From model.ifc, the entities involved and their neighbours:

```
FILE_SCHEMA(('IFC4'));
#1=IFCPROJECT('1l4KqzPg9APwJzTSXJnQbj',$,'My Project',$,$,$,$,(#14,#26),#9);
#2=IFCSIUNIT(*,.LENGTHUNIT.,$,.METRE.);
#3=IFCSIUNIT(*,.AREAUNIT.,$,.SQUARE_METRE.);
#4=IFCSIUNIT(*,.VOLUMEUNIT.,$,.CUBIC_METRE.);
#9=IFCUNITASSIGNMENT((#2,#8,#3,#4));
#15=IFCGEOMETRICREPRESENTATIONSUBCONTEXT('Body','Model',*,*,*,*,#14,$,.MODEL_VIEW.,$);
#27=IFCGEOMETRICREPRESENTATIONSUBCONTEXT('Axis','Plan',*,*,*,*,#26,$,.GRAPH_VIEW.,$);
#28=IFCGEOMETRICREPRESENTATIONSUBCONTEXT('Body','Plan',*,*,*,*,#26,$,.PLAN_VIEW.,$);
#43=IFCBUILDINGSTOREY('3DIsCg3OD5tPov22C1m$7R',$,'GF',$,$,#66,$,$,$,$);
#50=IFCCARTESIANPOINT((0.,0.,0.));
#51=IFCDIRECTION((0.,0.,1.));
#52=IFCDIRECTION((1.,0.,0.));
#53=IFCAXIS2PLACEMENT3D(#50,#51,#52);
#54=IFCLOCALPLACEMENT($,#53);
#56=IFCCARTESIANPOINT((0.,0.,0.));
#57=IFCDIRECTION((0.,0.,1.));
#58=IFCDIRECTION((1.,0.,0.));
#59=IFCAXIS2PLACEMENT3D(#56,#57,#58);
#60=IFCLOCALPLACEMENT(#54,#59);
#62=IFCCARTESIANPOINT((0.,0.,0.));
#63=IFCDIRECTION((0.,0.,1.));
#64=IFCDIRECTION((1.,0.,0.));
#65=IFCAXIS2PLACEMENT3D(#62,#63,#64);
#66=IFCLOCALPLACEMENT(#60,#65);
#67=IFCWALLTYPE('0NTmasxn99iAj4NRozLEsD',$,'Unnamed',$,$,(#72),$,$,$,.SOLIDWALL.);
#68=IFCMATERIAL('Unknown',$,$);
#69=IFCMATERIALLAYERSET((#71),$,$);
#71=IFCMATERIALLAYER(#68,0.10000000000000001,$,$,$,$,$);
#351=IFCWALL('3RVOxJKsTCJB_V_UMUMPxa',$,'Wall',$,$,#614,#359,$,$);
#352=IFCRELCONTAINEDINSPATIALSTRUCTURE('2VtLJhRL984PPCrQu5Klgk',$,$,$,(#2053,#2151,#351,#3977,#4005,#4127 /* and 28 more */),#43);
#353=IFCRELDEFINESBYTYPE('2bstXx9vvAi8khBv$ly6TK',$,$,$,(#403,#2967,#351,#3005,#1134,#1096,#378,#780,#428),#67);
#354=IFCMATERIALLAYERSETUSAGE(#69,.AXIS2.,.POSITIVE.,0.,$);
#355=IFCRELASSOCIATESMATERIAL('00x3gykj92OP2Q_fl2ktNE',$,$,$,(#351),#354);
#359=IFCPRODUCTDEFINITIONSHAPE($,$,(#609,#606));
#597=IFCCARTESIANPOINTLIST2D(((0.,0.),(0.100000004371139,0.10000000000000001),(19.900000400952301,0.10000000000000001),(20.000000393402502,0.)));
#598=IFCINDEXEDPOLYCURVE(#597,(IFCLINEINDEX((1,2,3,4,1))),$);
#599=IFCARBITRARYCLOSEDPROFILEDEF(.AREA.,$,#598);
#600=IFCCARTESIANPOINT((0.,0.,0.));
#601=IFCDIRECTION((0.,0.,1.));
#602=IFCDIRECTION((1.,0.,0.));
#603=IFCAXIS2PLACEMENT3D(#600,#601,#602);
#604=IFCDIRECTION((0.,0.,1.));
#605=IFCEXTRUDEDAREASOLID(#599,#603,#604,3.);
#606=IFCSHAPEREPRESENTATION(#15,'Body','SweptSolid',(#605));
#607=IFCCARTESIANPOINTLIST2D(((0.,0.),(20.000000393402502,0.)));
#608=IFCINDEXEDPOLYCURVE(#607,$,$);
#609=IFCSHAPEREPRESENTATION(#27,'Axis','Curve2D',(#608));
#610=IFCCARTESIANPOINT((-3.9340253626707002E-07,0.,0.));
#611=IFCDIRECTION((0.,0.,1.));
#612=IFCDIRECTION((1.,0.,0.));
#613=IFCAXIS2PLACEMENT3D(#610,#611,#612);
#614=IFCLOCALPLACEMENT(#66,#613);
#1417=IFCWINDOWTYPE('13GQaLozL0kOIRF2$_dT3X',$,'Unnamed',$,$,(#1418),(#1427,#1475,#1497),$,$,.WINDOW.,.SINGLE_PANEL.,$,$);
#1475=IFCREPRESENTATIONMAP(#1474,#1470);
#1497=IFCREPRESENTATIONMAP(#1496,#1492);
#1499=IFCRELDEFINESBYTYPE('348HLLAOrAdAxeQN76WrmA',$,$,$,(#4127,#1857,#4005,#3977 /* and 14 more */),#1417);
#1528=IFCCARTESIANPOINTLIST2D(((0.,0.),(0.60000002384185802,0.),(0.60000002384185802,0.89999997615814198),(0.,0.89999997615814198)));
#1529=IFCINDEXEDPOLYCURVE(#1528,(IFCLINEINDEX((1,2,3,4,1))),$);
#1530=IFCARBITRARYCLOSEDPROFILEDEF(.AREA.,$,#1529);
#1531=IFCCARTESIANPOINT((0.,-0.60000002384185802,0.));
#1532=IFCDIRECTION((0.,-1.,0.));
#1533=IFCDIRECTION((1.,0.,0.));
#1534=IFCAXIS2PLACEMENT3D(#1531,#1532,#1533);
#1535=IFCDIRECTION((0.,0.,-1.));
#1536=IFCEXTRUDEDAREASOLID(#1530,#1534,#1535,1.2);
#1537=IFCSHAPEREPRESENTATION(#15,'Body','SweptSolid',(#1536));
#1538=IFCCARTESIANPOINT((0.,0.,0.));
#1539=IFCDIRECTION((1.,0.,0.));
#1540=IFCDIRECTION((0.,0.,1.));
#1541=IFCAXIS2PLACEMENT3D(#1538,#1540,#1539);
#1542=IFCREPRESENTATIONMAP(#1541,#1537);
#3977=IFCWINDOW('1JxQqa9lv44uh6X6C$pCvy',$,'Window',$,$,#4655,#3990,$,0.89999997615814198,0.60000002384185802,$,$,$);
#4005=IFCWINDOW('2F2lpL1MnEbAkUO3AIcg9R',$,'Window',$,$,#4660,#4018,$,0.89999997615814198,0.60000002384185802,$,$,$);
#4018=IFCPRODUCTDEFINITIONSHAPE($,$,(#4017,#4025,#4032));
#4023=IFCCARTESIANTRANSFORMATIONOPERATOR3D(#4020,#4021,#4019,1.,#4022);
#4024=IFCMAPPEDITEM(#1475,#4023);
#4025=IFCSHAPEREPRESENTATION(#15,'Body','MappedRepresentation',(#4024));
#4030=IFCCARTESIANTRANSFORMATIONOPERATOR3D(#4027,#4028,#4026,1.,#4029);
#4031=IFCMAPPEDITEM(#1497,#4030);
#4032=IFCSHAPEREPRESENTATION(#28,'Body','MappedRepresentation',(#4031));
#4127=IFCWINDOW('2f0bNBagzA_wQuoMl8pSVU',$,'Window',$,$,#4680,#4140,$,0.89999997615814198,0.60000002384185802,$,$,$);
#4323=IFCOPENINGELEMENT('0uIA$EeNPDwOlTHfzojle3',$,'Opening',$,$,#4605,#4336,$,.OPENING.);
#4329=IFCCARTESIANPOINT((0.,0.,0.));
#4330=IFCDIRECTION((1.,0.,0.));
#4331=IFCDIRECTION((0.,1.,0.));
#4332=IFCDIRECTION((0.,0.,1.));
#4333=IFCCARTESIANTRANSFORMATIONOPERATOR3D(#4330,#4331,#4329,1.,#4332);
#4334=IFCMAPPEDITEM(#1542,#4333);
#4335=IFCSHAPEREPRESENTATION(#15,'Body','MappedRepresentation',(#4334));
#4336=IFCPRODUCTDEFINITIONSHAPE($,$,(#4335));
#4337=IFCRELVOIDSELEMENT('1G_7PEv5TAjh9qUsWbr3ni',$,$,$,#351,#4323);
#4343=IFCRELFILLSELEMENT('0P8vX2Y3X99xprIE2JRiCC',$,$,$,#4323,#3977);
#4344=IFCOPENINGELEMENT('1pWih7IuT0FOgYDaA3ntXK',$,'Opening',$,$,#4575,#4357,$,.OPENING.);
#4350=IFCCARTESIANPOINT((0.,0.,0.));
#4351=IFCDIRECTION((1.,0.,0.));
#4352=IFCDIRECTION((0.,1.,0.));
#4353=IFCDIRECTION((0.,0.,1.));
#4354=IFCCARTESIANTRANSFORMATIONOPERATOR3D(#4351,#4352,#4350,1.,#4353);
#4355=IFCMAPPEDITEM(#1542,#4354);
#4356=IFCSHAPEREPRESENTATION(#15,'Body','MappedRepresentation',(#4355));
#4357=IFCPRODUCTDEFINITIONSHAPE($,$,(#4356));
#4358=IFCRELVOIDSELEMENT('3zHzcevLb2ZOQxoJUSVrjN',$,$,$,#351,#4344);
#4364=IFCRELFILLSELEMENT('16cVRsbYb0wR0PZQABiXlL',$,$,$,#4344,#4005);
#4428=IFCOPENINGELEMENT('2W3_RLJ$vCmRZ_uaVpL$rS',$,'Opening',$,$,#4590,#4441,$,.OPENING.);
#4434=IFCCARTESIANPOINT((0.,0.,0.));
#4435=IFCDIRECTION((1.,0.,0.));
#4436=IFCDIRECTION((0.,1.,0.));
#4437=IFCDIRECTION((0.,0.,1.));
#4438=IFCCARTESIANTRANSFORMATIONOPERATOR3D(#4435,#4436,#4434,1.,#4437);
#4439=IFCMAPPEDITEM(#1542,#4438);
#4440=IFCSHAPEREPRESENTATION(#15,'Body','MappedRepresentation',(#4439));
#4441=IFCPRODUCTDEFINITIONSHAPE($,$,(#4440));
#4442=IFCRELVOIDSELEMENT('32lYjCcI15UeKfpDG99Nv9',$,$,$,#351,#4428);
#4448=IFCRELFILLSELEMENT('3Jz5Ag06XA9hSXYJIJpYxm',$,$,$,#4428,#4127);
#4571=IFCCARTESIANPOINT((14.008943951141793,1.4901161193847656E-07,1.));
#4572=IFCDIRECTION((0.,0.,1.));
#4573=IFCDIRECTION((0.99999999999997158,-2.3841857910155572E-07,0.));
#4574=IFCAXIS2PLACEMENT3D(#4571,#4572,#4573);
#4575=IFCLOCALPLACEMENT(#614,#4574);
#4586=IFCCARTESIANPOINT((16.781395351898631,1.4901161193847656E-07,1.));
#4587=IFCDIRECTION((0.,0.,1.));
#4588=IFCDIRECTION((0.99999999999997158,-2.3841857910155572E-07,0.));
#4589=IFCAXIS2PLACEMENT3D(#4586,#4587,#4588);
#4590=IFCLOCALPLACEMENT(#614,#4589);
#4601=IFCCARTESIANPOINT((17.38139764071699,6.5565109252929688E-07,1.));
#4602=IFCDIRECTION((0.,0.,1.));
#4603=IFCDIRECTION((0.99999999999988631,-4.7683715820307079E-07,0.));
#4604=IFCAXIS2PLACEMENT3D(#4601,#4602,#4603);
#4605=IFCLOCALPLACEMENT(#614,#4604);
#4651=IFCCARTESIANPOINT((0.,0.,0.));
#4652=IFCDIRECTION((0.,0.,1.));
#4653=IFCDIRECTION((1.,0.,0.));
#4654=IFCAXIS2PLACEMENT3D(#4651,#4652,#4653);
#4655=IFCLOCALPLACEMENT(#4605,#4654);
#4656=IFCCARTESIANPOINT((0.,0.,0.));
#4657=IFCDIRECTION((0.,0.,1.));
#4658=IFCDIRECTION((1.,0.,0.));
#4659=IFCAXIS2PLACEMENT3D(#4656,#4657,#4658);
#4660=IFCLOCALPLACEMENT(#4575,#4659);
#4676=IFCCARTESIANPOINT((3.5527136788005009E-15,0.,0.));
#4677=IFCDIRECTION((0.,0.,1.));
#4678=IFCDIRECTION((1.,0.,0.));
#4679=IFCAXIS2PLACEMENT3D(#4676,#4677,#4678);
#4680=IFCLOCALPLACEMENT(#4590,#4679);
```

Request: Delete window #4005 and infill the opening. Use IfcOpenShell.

```python
import ifcopenshell
import ifcopenshell.api.feature
import ifcopenshell.api.root
import ifcopenshell.geom
import ifcopenshell.util.shape

model = ifcopenshell.open("model.ifc")
settings = ifcopenshell.geom.settings()


def volume(element):
    """Net volume in cubic metres, openings subtracted."""
    shape = ifcopenshell.geom.create_shape(settings, element)
    return ifcopenshell.util.shape.get_volume(shape.geometry)


window = model.by_guid("2F2lpL1MnEbAkUO3AIcg9R")
opening = window.FillsVoids[0].RelatingOpeningElement
wall = opening.VoidsElements[0].RelatingBuildingElement
before = volume(wall)

ifcopenshell.api.root.remove_product(model, product=window)
ifcopenshell.api.feature.remove_feature(model, feature=opening)

after = volume(wall)

print(f"wall volume {before:.3f} -> {after:.3f} m3")

model.write("model_edited.ifc")
```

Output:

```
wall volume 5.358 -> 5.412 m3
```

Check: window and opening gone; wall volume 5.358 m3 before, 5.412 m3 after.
